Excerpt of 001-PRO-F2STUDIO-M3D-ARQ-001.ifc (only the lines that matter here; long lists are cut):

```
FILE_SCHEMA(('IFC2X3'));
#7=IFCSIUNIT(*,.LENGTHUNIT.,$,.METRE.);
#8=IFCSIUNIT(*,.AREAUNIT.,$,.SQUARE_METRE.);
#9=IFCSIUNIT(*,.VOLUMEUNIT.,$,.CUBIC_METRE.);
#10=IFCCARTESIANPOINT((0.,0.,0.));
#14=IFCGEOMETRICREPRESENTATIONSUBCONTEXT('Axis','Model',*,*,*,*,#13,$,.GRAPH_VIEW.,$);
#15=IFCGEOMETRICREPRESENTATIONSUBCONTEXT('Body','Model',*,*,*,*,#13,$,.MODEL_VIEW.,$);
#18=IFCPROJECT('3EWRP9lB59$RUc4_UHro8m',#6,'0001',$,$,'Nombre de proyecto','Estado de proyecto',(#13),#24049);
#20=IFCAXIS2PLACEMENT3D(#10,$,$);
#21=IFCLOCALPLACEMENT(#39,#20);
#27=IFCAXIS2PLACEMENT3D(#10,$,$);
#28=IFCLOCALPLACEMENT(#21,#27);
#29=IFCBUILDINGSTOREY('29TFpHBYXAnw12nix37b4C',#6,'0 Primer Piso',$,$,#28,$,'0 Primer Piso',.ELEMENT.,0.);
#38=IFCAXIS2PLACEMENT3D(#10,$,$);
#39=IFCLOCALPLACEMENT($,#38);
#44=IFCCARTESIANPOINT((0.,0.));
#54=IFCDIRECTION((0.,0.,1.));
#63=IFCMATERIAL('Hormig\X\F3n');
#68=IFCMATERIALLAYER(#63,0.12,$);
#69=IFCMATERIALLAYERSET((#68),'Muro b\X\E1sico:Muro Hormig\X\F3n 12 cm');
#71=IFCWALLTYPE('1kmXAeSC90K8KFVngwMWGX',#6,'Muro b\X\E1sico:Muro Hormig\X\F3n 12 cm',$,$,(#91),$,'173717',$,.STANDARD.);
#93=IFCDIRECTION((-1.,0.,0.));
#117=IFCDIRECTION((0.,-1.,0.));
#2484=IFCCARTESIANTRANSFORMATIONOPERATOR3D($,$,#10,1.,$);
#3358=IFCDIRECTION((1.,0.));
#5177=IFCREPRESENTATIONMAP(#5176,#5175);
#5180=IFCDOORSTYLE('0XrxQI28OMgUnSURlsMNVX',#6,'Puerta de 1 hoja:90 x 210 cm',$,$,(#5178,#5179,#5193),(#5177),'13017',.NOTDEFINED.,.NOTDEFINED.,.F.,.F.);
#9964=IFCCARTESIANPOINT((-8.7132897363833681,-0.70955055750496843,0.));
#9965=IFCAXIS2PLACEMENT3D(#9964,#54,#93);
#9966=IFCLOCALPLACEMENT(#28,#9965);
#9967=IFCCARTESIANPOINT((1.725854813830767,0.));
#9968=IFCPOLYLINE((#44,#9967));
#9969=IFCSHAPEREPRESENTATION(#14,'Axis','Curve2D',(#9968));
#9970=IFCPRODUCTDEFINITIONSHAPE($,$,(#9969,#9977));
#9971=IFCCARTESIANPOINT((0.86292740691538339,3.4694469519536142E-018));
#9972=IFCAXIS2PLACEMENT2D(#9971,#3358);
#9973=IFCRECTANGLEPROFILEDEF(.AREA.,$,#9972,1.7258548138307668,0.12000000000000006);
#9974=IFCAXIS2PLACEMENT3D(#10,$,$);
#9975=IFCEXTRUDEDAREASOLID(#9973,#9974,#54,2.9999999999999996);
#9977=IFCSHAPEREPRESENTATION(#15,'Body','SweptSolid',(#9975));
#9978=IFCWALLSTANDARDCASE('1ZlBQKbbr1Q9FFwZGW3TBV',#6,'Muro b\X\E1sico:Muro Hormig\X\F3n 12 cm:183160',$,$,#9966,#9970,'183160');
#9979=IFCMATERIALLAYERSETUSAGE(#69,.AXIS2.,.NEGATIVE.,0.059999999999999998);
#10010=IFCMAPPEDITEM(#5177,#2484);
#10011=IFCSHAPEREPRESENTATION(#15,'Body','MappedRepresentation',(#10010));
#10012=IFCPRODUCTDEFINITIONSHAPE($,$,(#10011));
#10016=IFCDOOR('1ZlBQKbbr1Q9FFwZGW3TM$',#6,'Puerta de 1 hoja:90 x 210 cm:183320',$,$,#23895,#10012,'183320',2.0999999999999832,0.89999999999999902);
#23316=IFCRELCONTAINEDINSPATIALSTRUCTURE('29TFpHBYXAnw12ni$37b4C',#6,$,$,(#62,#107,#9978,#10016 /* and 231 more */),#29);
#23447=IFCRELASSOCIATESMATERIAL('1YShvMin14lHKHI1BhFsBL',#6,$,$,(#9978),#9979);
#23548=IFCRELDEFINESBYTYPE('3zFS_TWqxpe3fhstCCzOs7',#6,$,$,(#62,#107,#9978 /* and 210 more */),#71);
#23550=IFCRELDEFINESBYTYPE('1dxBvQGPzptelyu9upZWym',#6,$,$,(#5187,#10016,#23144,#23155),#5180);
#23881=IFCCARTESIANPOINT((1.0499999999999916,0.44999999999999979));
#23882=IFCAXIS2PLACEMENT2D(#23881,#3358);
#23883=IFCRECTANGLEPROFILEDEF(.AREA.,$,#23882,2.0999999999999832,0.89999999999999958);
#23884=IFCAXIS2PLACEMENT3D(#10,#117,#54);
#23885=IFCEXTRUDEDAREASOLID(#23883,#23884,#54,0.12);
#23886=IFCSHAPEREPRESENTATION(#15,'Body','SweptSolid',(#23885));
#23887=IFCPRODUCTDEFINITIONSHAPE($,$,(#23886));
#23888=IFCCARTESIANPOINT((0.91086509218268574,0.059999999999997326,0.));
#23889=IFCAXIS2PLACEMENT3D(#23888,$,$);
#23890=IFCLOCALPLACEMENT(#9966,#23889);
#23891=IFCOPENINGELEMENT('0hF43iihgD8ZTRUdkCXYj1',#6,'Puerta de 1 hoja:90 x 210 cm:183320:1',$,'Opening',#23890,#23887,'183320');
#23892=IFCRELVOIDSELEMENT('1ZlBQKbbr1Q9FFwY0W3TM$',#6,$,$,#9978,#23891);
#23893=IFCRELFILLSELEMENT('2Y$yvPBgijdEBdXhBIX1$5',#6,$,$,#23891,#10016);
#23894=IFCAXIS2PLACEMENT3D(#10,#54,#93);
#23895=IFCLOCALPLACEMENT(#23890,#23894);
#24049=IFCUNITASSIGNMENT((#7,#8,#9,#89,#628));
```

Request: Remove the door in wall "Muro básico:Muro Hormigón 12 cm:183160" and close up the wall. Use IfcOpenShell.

```python
import ifcopenshell
import ifcopenshell.api.feature
import ifcopenshell.api.root
import ifcopenshell.geom
import ifcopenshell.util.shape

model = ifcopenshell.open("001-PRO-F2STUDIO-M3D-ARQ-001.ifc")
settings = ifcopenshell.geom.settings()


def volume(element):
    """Net volume in cubic metres, openings subtracted."""
    shape = ifcopenshell.geom.create_shape(settings, element)
    return ifcopenshell.util.shape.get_volume(shape.geometry)


door = model.by_guid("1ZlBQKbbr1Q9FFwZGW3TM$")
opening = door.FillsVoids[0].RelatingOpeningElement
wall = opening.VoidsElements[0].RelatingBuildingElement
before = volume(wall)

ifcopenshell.api.root.remove_product(model, product=door)
ifcopenshell.api.feature.remove_feature(model, feature=opening)

after = volume(wall)

print(f"wall volume {before:.3f} -> {after:.3f} m3")

model.write("001-PRO-F2STUDIO-M3D-ARQ-001_edited.ifc")
```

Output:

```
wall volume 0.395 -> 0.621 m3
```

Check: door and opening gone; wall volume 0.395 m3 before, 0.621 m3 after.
